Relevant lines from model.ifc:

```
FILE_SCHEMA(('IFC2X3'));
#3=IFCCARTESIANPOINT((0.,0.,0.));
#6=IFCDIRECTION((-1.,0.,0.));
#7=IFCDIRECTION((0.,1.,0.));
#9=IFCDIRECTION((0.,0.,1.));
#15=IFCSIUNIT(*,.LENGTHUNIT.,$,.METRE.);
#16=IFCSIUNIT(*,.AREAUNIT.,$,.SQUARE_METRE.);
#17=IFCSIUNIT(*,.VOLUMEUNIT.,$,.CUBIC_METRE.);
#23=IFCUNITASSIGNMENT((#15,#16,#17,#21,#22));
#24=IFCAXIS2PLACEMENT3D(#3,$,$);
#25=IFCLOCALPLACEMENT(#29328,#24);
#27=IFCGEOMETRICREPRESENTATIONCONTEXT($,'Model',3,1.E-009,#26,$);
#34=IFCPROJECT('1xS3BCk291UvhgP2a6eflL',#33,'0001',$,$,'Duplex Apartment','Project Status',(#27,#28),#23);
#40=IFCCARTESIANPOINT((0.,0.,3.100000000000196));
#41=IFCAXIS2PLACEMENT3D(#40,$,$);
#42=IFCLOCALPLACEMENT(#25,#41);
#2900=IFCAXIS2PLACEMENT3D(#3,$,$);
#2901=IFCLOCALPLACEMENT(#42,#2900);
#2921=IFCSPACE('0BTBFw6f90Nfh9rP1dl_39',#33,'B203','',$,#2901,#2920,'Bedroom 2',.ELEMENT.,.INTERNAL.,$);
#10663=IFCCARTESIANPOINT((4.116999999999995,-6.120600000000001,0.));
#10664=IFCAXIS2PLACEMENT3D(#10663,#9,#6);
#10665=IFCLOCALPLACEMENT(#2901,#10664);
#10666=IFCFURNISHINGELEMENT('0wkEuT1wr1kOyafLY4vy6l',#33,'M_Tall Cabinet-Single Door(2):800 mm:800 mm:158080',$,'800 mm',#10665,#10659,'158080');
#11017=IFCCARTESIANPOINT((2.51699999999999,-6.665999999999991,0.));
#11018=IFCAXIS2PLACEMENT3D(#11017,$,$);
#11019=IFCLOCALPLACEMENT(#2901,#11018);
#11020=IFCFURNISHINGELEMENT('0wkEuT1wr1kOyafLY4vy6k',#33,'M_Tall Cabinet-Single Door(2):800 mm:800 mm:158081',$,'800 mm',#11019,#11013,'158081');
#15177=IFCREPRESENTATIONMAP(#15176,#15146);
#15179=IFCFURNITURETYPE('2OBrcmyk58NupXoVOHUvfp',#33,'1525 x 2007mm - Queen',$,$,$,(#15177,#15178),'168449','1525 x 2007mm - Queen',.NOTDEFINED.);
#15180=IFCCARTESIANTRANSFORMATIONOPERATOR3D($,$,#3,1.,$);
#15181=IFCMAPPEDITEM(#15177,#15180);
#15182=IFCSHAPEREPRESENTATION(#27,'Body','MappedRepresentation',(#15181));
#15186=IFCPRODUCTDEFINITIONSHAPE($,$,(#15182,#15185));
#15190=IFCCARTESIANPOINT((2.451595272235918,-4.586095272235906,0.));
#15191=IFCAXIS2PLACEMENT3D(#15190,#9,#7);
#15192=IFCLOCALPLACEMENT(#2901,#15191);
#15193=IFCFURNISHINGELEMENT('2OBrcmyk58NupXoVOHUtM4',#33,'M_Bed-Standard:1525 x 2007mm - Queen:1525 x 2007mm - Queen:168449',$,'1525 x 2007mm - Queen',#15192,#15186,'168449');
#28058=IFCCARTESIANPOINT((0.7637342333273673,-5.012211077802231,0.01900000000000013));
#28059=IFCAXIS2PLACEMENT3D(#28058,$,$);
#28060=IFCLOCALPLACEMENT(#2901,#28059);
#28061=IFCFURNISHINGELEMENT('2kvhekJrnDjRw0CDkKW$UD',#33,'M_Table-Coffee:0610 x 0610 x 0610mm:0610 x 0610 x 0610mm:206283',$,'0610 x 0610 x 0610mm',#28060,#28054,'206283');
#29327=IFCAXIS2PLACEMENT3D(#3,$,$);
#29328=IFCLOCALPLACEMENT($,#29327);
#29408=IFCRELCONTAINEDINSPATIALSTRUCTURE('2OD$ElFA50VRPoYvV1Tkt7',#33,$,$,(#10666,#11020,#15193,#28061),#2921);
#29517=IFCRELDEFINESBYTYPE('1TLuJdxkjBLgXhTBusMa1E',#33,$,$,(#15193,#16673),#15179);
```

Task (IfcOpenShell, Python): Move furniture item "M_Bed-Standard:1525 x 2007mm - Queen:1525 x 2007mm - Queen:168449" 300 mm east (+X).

```python
import ifcopenshell
import ifcopenshell.api.geometry
import ifcopenshell.util.placement
import ifcopenshell.util.unit

model = ifcopenshell.open("model.ifc")
unit_scale = ifcopenshell.util.unit.calculate_unit_scale(model)

item = model.by_guid("2OBrcmyk58NupXoVOHUtM4")
matrix = ifcopenshell.util.placement.get_local_placement(item.ObjectPlacement)
matrix[0, 3] += 0.3 / unit_scale
ifcopenshell.api.geometry.edit_object_placement(model, product=item, matrix=matrix, is_si=False)

print(ifcopenshell.util.placement.get_local_placement(item.ObjectPlacement).round(3) + 0.0)

model.write("model_edited.ifc")
```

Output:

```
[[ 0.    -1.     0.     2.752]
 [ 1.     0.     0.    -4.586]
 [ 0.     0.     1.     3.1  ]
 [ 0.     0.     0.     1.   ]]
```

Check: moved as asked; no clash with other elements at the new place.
